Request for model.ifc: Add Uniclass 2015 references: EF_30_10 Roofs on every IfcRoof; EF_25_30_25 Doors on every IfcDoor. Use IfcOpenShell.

First a look at what the model holds.

```python
import ifcopenshell

model = ifcopenshell.open("model.ifc")
print(model.schema)
print("classifications:", [c.Name for c in model.by_type("IfcClassification")])
for ifc_class in ("IfcDoor", "IfcRoof", "IfcStair", "IfcWall", "IfcWindow"):
    print(ifc_class, len(model.by_type(ifc_class)))
```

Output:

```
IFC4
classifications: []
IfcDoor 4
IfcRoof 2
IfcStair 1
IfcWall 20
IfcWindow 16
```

```python
import ifcopenshell
import ifcopenshell.api.classification

model = ifcopenshell.open("model.ifc")

system = ifcopenshell.api.classification.add_classification(model, classification="Uniclass 2015")

codes = {
    "IfcRoof": ("EF_30_10", "Roofs"),
    "IfcDoor": ("EF_25_30_25", "Doors"),
}
for ifc_class, (code, name) in codes.items():
    products = model.by_type(ifc_class)
    ifcopenshell.api.classification.add_reference(
        model, products=products, classification=system, identification=code, name=name
    )
    print(code, len(products))

model.write("model_v2.ifc")
```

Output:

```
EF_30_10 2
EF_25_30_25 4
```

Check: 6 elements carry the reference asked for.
